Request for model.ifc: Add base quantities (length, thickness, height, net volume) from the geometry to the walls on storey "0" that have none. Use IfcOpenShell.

First a look at what the model holds.

```python
import ifcopenshell
import ifcopenshell.util.element
import ifcopenshell.util.unit

model = ifcopenshell.open("model.ifc")
print(model.schema)
for unit_type in ("LENGTHUNIT", "AREAUNIT", "VOLUMEUNIT"):
    print(unit_type, ifcopenshell.util.unit.calculate_unit_scale(model, unit_type))
storey = next(s for s in model.by_type("IfcBuildingStorey") if s.Name == "0")
walls = [e for e in ifcopenshell.util.element.get_decomposition(storey) if e.is_a("IfcWall")]
for e in sorted(walls, key=lambda e: e.id()):
    print(e.id(), e.is_a(), e.Name, list(ifcopenshell.util.element.get_psets(e, qtos_only=True)), sep=" | ")
```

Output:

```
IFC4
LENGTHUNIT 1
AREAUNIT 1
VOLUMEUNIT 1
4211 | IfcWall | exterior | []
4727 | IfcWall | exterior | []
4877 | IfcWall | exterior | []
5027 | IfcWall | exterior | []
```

```python
import ifcopenshell
import ifcopenshell.api.pset
import ifcopenshell.geom
import ifcopenshell.util.element
import ifcopenshell.util.shape
import ifcopenshell.util.unit

model = ifcopenshell.open("model.ifc")
unit_scale = ifcopenshell.util.unit.calculate_unit_scale(model)
volume_scale = ifcopenshell.util.unit.calculate_unit_scale(model, "VOLUMEUNIT")
settings = ifcopenshell.geom.settings()

storey = next(s for s in model.by_type("IfcBuildingStorey") if s.Name == "0")
walls = [e for e in ifcopenshell.util.element.get_decomposition(storey) if e.is_a("IfcWall")]

for e in sorted(walls, key=lambda e: e.id()):
    if ifcopenshell.util.element.get_psets(e, qtos_only=True, should_inherit=False):
        continue
    # Geometry comes back in metres, in the element's own axes.
    shape = ifcopenshell.geom.create_shape(settings, e)
    values = {
        "Length": ifcopenshell.util.shape.get_x(shape.geometry) / unit_scale,
        "Width": ifcopenshell.util.shape.get_y(shape.geometry) / unit_scale,
        "Height": ifcopenshell.util.shape.get_z(shape.geometry) / unit_scale,
        "NetVolume": ifcopenshell.util.shape.get_volume(shape.geometry) / volume_scale,
    }
    qto = ifcopenshell.api.pset.add_qto(model, product=e, name="Qto_WallBaseQuantities")
    ifcopenshell.api.pset.edit_qto(model, qto=qto, properties=values)
    print(e.id(), {k: round(v, 3) for k, v in values.items()})

model.write("model-out.ifc")
```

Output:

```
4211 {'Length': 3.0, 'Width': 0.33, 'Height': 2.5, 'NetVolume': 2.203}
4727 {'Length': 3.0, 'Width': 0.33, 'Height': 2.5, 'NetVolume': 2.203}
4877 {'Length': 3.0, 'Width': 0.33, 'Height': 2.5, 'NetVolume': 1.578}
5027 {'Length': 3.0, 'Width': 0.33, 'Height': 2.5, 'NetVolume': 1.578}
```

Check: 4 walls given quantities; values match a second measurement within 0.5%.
